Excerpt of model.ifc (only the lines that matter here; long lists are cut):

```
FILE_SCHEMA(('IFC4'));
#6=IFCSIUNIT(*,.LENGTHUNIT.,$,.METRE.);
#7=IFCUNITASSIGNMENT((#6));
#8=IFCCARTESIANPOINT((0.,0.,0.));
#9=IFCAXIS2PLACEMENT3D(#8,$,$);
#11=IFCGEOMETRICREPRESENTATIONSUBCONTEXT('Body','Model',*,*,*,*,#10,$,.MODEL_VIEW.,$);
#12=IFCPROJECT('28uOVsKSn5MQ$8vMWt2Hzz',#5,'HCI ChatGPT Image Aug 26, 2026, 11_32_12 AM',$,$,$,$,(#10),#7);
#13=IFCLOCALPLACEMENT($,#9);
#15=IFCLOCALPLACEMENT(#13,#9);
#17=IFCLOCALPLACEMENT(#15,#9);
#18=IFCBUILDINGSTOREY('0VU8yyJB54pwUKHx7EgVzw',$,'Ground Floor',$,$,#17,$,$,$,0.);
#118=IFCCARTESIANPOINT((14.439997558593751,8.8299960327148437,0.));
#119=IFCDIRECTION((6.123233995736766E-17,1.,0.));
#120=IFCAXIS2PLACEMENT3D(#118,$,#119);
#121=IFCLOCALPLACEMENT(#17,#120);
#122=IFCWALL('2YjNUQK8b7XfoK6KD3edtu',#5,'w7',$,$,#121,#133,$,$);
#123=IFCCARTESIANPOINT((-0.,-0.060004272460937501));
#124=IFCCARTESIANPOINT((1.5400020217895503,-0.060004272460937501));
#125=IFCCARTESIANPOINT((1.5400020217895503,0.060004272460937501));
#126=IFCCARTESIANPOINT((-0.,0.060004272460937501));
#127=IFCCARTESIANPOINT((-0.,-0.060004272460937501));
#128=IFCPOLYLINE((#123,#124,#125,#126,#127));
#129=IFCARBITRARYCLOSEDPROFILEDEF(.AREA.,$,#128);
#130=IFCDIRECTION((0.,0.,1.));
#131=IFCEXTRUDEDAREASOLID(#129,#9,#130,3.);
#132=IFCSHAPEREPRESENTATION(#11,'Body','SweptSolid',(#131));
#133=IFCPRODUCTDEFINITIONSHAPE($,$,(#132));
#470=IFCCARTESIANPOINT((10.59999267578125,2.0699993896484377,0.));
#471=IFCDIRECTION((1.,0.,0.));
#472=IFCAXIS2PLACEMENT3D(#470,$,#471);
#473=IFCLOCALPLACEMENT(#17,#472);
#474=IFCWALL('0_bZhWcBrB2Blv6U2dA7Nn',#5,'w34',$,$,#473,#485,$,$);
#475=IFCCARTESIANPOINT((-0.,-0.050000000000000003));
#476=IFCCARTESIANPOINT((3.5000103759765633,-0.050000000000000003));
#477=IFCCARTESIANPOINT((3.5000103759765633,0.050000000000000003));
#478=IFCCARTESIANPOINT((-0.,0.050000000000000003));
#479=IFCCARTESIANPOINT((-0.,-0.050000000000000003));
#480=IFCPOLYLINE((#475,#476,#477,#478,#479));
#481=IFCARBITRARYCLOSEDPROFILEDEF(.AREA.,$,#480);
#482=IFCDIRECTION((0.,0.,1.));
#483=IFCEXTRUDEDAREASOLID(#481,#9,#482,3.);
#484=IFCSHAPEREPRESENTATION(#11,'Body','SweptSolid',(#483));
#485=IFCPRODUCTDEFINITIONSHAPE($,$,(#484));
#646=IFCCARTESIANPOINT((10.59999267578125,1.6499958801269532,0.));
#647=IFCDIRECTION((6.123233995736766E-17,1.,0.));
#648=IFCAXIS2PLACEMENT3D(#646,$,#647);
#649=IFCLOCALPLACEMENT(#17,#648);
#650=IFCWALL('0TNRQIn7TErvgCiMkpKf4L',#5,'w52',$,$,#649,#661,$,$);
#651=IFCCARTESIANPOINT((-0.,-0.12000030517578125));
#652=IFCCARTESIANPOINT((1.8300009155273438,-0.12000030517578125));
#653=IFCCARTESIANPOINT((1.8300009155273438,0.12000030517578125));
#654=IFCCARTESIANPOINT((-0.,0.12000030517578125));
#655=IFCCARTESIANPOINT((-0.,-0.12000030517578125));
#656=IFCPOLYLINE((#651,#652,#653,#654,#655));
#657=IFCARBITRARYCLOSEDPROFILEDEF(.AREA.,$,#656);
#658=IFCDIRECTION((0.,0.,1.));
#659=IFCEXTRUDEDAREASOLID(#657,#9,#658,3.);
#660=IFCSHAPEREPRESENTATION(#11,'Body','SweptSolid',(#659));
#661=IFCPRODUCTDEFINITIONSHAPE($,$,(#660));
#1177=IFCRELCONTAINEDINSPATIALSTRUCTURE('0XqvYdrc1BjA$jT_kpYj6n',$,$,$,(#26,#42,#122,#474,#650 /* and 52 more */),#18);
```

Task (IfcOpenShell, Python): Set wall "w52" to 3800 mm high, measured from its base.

```python
import ifcopenshell
import ifcopenshell.geom
import ifcopenshell.util.representation
import ifcopenshell.util.shape
import ifcopenshell.util.unit

model = ifcopenshell.open("model.ifc")
unit_scale = ifcopenshell.util.unit.calculate_unit_scale(model)
settings = ifcopenshell.geom.settings()


def volume(element):
    """Net volume in cubic metres, openings subtracted."""
    shape = ifcopenshell.geom.create_shape(settings, element)
    return ifcopenshell.util.shape.get_volume(shape.geometry)


wall = model.by_id(650)
before = volume(wall)

body = ifcopenshell.util.representation.get_representation(wall, "Model", "Body")
solid = body.Items[0]
old_height = solid.Depth
solid.Depth = 3.8 / unit_scale
after = volume(wall)

print(f"height {old_height:g} -> {solid.Depth:g}, volume {before:.3f} -> {after:.3f} m3")

model.write("model-out.ifc")
```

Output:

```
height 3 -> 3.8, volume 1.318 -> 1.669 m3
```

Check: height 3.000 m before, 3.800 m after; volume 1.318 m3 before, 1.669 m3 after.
